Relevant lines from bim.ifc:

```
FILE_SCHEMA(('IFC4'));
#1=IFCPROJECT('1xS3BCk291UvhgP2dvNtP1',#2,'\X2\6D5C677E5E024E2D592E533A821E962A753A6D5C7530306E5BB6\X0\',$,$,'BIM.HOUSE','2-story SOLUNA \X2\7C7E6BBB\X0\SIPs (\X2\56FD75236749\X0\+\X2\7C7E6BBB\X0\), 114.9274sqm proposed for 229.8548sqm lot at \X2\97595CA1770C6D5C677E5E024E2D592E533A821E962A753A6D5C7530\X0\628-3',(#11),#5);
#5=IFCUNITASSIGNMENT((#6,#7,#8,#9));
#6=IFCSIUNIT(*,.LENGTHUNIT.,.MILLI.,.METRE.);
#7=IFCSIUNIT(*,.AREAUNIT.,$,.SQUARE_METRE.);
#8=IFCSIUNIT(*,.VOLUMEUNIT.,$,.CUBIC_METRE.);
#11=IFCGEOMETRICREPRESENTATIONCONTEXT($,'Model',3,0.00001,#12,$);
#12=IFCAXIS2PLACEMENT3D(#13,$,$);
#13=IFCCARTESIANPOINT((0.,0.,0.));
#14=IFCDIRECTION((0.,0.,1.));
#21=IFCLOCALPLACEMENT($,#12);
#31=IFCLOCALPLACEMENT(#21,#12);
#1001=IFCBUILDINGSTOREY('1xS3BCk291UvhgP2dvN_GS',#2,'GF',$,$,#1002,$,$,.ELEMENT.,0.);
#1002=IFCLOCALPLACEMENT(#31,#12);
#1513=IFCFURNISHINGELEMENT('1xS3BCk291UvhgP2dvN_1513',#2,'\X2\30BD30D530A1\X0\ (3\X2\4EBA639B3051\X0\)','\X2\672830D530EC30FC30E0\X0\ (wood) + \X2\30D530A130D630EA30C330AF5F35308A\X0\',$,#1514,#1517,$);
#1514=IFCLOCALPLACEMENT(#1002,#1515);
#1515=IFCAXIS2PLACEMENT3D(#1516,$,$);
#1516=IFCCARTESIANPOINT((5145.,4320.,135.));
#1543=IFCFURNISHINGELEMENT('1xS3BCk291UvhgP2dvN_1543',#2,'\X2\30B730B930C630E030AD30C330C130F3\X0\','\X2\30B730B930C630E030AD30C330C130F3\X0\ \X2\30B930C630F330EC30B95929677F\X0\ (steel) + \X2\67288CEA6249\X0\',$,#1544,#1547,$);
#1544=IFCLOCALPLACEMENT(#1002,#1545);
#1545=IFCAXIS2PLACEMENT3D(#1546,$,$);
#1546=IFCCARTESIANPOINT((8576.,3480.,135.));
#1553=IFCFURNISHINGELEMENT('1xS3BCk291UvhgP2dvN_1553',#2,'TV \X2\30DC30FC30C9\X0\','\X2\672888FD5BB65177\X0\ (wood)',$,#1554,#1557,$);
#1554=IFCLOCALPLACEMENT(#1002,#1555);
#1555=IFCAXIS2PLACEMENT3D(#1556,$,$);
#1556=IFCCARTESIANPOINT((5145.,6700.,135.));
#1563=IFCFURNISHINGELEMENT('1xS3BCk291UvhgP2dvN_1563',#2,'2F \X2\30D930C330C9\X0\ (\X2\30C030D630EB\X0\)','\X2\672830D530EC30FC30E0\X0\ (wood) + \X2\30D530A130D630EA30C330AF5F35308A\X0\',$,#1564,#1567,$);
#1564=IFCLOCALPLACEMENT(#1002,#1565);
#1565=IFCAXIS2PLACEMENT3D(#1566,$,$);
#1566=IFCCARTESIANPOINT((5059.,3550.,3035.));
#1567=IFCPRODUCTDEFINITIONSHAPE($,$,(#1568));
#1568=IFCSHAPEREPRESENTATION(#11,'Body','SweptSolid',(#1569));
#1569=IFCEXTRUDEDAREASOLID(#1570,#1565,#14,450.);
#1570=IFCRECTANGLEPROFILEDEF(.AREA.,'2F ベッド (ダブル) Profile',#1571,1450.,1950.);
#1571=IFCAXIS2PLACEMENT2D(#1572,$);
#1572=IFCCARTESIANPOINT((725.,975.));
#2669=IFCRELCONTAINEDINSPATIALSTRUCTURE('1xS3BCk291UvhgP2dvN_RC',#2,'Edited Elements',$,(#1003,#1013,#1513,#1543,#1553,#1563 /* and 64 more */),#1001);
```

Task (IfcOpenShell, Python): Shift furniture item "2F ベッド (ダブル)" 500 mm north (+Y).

```python
import ifcopenshell
import ifcopenshell.api.geometry
import ifcopenshell.util.placement
import ifcopenshell.util.unit

model = ifcopenshell.open("bim.ifc")
unit_scale = ifcopenshell.util.unit.calculate_unit_scale(model)

item = model.by_id(1563)
matrix = ifcopenshell.util.placement.get_local_placement(item.ObjectPlacement)
matrix[1, 3] += 0.5 / unit_scale
ifcopenshell.api.geometry.edit_object_placement(model, product=item, matrix=matrix, is_si=False)

print(ifcopenshell.util.placement.get_local_placement(item.ObjectPlacement).round(3) + 0.0)

model.write("bim_updated.ifc")
```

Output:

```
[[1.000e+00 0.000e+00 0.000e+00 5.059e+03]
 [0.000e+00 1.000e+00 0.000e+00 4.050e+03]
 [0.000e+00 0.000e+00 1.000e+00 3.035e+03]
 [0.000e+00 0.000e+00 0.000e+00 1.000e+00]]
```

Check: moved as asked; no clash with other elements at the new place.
